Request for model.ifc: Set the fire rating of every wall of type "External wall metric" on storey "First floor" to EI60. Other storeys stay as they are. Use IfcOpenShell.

First a look at what the model holds.

```python
import ifcopenshell
import ifcopenshell.util.element

model = ifcopenshell.open("model.ifc")
print(model.schema)
storey = next(s for s in model.by_type("IfcBuildingStorey") if s.Name == "First floor")
walls = [e for e in ifcopenshell.util.element.get_decomposition(storey) if e.is_a("IfcWall")]
seen = {}
for e in walls:
    element_type = ifcopenshell.util.element.get_type(e)
    key = (element_type.Name if element_type != e and element_type else None, ifcopenshell.util.element.get_pset(e, "Pset_WallCommon", "FireRating"))
    seen[key] = seen.get(key, 0) + 1
for (name, value), count in sorted(seen.items(), key=str):
    print(count, "x", name, "|", value)
```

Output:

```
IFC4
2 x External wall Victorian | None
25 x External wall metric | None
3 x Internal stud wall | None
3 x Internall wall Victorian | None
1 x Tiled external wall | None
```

```python
import ifcopenshell
import ifcopenshell.api.pset
import ifcopenshell.util.element

model = ifcopenshell.open("model.ifc")

storey = next(s for s in model.by_type("IfcBuildingStorey") if s.Name == "First floor")
walls = [e for e in ifcopenshell.util.element.get_decomposition(storey) if e.is_a("IfcWall")]

count = 0
for e in walls:
    element_type = ifcopenshell.util.element.get_type(e)
    if element_type in (None, e) or element_type.Name != "External wall metric":
        continue
    # add_pset returns the element's existing set when there is one.
    pset = ifcopenshell.api.pset.add_pset(model, product=e, name="Pset_WallCommon")
    ifcopenshell.api.pset.edit_pset(model, pset=pset, properties={"FireRating": "EI60"})
    count += 1

print(count, "walls updated")

model.write("model_v2.ifc")
```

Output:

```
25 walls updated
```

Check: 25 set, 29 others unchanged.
